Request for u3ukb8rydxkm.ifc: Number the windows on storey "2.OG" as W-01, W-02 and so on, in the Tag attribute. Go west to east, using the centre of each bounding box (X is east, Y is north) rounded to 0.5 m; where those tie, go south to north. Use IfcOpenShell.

First a look at what the model holds.

```python
import ifcopenshell
import ifcopenshell.util.element
import ifcopenshell.util.placement

model = ifcopenshell.open("u3ukb8rydxkm.ifc")
print(model.schema)
storey = next(s for s in model.by_type("IfcBuildingStorey") if s.Name == "2.OG")
windows = [e for e in ifcopenshell.util.element.get_decomposition(storey) if e.is_a("IfcWindow")]
for e in sorted(windows, key=lambda e: e.id()):
    origin = ifcopenshell.util.placement.get_local_placement(e.ObjectPlacement)[:3, 3]
    print(e.id(), e.Tag, e.Name, origin.round(2) + 0.0, sep=" | ")
```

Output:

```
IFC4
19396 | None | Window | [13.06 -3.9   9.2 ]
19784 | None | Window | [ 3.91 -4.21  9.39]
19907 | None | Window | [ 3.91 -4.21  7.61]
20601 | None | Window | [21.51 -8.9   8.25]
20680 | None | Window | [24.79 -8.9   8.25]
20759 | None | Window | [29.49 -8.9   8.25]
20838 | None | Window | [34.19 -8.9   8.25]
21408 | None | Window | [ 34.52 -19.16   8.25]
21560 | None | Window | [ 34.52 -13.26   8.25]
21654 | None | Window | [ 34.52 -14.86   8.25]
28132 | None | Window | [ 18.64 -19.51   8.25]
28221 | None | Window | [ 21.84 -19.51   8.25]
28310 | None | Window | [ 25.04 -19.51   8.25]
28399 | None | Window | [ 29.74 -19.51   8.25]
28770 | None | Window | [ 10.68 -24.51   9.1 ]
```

```python
import ifcopenshell
import ifcopenshell.geom
import ifcopenshell.util.element
import ifcopenshell.util.shape

model = ifcopenshell.open("u3ukb8rydxkm.ifc")
settings = ifcopenshell.geom.settings()
settings.set("use-world-coords", True)


def centre(element):
    shape = ifcopenshell.geom.create_shape(settings, element)
    return ifcopenshell.util.shape.get_bbox_centroid(shape.geometry)


storey = next(s for s in model.by_type("IfcBuildingStorey") if s.Name == "2.OG")
windows = [e for e in ifcopenshell.util.element.get_decomposition(storey) if e.is_a("IfcWindow")]

# Insertion points can sit at a corner or the storey origin, so sort by the geometry (in metres).
centres = {e: centre(e) for e in windows}
windows.sort(key=lambda e: (round(centres[e][0] / 0.5), centres[e][1]))

for i, e in enumerate(windows, start=1):
    number = f"W-{i:02d}"
    e.Tag = number
    print(e.id(), number)

model.write("u3ukb8rydxkm_v2.ifc")
```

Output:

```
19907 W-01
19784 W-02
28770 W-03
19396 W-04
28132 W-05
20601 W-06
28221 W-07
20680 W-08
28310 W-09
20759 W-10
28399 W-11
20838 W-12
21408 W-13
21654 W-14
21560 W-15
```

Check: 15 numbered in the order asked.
